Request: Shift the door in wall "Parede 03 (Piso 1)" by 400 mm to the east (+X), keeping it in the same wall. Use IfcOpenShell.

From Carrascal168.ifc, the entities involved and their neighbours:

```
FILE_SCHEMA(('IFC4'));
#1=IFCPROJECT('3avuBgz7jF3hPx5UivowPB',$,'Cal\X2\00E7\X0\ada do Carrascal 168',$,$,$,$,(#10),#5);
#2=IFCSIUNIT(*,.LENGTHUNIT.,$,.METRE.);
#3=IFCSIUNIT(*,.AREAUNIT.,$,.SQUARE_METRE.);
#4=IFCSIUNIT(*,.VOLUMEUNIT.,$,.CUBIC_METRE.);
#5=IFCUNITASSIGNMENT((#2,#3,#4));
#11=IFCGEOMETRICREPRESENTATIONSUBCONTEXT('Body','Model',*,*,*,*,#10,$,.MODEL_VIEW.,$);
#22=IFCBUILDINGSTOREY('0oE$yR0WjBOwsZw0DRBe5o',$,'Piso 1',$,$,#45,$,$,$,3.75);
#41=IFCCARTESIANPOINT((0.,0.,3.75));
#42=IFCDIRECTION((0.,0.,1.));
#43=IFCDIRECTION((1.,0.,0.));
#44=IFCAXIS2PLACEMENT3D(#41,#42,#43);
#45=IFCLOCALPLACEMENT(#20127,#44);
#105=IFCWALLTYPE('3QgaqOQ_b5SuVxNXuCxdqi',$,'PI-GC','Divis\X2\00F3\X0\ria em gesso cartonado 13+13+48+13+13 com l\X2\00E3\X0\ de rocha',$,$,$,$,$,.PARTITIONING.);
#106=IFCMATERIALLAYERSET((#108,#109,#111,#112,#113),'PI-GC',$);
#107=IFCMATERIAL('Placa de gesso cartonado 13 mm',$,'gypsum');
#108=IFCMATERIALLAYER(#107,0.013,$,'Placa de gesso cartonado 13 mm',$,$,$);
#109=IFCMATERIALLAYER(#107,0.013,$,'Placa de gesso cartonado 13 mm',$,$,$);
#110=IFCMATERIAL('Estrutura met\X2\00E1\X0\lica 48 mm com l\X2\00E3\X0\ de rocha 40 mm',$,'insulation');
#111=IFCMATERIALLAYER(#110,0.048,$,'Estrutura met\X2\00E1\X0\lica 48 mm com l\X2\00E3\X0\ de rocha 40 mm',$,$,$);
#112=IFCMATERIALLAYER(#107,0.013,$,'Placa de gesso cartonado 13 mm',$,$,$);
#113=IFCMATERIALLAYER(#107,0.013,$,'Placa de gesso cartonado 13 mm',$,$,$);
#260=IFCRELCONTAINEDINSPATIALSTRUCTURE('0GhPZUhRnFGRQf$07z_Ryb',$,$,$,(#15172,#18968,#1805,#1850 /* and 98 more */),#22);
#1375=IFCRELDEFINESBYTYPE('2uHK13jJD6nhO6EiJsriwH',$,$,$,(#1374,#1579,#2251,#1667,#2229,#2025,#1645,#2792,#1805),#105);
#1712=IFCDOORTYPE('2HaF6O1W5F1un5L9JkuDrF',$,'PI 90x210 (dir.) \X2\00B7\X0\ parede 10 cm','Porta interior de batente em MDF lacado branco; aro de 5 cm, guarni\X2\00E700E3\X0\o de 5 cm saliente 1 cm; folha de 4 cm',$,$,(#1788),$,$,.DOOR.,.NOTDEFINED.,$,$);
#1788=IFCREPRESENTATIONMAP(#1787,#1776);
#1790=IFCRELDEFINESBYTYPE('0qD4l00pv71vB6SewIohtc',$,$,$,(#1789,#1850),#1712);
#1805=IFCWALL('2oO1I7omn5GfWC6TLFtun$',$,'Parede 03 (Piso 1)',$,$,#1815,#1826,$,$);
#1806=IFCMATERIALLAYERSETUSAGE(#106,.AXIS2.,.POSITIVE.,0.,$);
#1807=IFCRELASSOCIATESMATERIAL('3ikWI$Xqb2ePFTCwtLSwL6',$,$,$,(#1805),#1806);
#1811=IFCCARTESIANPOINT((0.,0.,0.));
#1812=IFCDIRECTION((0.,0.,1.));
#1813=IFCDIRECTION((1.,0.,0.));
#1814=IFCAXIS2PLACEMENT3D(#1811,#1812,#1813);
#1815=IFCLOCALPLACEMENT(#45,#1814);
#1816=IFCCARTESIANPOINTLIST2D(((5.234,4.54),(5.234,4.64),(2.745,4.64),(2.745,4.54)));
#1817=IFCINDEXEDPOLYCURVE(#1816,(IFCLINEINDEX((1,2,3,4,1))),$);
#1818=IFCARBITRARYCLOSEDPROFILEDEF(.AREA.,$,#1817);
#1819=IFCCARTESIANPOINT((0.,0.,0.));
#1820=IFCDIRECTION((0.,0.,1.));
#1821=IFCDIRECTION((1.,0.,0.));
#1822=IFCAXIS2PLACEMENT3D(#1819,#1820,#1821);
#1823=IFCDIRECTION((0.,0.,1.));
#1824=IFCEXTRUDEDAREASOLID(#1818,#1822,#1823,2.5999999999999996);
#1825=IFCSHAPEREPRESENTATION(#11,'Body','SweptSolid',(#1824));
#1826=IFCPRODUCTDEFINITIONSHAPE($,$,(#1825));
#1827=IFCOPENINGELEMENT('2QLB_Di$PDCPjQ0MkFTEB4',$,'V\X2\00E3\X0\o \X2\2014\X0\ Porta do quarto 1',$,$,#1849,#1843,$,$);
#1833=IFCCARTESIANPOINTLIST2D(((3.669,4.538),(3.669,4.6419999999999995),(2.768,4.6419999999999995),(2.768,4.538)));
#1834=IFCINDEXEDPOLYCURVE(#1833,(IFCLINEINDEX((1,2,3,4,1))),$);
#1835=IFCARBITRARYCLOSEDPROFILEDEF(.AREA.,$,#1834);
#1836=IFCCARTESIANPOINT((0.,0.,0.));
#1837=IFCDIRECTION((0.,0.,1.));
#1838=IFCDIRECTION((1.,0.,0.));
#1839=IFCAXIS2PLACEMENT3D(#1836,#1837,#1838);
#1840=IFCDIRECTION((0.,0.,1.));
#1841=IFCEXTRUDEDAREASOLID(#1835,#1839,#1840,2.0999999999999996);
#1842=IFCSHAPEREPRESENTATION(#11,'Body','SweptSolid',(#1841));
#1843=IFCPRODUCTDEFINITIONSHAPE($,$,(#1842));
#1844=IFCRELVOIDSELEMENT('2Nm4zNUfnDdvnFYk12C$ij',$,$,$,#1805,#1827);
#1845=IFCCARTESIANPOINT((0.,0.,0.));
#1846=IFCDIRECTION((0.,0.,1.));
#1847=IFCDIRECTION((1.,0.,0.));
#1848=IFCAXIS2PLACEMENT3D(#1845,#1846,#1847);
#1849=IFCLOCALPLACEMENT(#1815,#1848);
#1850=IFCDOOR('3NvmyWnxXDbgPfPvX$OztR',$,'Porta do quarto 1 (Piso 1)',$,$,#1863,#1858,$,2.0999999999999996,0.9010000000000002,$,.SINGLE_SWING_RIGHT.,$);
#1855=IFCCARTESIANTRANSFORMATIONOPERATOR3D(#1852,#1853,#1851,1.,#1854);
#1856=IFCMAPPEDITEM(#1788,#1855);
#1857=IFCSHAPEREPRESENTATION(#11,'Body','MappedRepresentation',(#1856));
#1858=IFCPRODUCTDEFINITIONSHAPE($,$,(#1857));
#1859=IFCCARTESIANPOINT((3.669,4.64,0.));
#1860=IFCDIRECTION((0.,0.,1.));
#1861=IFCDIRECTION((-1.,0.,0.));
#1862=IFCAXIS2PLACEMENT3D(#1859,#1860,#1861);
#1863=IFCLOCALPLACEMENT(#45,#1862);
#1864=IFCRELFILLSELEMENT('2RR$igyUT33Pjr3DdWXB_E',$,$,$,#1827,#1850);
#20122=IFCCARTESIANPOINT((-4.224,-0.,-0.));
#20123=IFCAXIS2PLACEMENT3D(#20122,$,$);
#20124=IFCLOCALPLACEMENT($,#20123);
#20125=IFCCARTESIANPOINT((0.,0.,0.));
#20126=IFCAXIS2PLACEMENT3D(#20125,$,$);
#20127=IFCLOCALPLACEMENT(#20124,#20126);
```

```python
import ifcopenshell
import ifcopenshell.api.geometry
import ifcopenshell.util.placement

model = ifcopenshell.open("Carrascal168.ifc")

door = model.by_guid("3NvmyWnxXDbgPfPvX$OztR")
opening = door.FillsVoids[0].RelatingOpeningElement
wall = opening.VoidsElements[0].RelatingBuildingElement

wall_matrix = ifcopenshell.util.placement.get_local_placement(wall.ObjectPlacement)
shift = wall_matrix[:3, 0] * 0.4
before = ifcopenshell.util.placement.get_local_placement(door.ObjectPlacement)[:3, 3].copy()

# The door is not placed relative to its opening, so move both.
for product in (opening, door):
    matrix = ifcopenshell.util.placement.get_local_placement(product.ObjectPlacement)
    matrix[:3, 3] += shift
    ifcopenshell.api.geometry.edit_object_placement(model, product=product, matrix=matrix, is_si=False)

after = ifcopenshell.util.placement.get_local_placement(door.ObjectPlacement)[:3, 3]
print("door moved by", (after - before).round(3) + 0.0)

model.write("Carrascal168_v2.ifc")
```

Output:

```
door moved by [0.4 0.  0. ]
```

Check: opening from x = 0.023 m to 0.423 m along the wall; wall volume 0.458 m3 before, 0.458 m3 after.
